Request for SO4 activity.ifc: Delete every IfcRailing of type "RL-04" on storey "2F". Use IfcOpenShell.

First a look at what the model holds.

```python
import ifcopenshell
import ifcopenshell.util.element

model = ifcopenshell.open("SO4 activity.ifc")
print(model.schema)
storey = next(s for s in model.by_type("IfcBuildingStorey") if s.Name == "2F")
railings = [e for e in ifcopenshell.util.element.get_decomposition(storey) if e.is_a("IfcRailing")]
seen = {}
for e in railings:
    element_type = ifcopenshell.util.element.get_type(e)
    name = element_type.Name if element_type not in (None, e) else None
    seen[name] = seen.get(name, 0) + 1
for name, count in sorted(seen.items(), key=str):
    print(count, "x", name)
```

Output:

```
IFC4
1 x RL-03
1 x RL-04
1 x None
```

```python
import ifcopenshell
import ifcopenshell.api.root
import ifcopenshell.util.element

model = ifcopenshell.open("SO4 activity.ifc")

storey = next(s for s in model.by_type("IfcBuildingStorey") if s.Name == "2F")
railings = [e for e in ifcopenshell.util.element.get_decomposition(storey) if e.is_a("IfcRailing")]
targets = [e for e in railings if (t := ifcopenshell.util.element.get_type(e)) not in (None, e) and t.Name == "RL-04"]

for e in targets:
    ifcopenshell.api.root.remove_product(model, product=e)
print(len(targets), "removed")

model.write("SO4 activity_updated.ifc")
```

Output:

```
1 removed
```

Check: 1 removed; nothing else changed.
